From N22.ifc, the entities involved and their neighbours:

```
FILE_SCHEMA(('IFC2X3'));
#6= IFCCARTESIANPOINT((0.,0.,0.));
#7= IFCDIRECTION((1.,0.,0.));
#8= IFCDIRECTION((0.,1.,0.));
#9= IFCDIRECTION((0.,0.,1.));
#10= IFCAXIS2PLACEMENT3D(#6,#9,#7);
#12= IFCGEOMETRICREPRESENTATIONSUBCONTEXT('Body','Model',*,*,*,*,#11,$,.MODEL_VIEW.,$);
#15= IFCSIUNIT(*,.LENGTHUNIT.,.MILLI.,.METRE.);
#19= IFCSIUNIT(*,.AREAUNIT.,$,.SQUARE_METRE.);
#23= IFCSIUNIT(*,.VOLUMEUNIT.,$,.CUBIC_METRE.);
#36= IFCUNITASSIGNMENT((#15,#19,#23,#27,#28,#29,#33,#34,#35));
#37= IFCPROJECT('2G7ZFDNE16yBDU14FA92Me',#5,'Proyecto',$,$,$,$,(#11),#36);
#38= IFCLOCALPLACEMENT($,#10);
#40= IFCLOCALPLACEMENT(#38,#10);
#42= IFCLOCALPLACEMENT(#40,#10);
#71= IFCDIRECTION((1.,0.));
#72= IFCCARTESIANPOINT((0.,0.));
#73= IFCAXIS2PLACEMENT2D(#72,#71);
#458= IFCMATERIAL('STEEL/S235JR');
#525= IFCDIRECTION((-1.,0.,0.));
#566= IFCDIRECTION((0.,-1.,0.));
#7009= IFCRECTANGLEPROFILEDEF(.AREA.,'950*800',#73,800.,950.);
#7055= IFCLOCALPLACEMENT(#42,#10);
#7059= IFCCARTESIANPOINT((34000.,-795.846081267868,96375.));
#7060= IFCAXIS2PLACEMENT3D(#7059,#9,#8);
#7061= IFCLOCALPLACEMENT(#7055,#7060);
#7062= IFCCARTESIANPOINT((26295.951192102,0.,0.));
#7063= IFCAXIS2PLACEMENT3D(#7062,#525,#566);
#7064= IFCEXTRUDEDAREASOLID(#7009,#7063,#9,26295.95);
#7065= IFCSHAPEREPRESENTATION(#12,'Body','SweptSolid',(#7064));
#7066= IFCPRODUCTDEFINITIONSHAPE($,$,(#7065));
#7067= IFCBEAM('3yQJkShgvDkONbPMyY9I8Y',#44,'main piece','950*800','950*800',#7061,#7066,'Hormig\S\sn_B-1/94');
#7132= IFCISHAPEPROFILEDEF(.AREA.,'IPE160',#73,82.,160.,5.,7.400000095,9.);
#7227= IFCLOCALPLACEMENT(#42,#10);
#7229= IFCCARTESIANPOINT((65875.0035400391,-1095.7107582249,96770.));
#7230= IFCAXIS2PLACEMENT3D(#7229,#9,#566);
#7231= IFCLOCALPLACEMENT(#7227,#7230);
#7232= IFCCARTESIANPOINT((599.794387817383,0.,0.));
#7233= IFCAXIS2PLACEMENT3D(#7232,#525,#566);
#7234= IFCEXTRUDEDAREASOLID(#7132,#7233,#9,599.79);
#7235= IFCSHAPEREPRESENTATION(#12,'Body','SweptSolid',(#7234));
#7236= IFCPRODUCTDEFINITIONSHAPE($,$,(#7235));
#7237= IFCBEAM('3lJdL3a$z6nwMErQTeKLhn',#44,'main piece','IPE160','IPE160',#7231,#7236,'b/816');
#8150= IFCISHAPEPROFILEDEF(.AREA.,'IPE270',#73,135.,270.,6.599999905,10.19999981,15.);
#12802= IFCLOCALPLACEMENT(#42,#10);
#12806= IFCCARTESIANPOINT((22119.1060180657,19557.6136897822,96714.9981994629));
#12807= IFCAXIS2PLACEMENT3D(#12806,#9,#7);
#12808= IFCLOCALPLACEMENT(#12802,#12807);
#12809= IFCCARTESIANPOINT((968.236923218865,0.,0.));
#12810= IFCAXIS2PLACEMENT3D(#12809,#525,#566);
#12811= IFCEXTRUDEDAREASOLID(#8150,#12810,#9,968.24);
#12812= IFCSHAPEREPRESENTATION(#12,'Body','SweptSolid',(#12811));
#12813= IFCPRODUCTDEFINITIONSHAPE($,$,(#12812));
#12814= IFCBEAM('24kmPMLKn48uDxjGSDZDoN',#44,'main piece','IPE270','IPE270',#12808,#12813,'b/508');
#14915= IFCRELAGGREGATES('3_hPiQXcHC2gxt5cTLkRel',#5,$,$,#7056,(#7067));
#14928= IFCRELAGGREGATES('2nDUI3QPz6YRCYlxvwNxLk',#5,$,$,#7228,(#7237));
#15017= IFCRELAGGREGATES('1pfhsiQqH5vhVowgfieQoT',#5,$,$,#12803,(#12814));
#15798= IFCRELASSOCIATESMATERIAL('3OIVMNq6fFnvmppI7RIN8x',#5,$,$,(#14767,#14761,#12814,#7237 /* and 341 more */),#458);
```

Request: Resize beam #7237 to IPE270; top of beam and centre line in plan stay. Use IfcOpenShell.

```python
import ifcopenshell
import ifcopenshell.util.element
import ifcopenshell.util.representation

model = ifcopenshell.open("N22.ifc")

member = model.by_guid("3lJdL3a$z6nwMErQTeKLhn")
source = next(p for p in model.by_type("IfcIShapeProfileDef") if p.ProfileName == "IPE270")

body = ifcopenshell.util.representation.get_representation(member, "Model", "Body")
solid = body.Items[0]
old_profile = solid.SweptArea

# Copy the section's sizes but keep this member's own profile position.
profile = ifcopenshell.util.element.copy(model, source)
# Profiles are centred, so shift by half the change in depth to hold the top.
shift = (old_profile.OverallDepth - profile.OverallDepth) / 2
x, y = old_profile.Position.Location.Coordinates
up = (0.0, 1.0)  # upwards, in the solid's own plane
location = model.createIfcCartesianPoint((x + up[0] * shift, y + up[1] * shift))
profile.Position = model.createIfcAxis2Placement2D(location, old_profile.Position.RefDirection)
solid.SweptArea = profile
if not model.get_total_inverses(old_profile):
    ifcopenshell.util.element.remove_deep2(model, old_profile)
member.Description = member.Description.replace("IPE160", "IPE270")
member.ObjectType = member.ObjectType.replace("IPE160", "IPE270")

print(solid.SweptArea)

model.write("N22-out.ifc")
```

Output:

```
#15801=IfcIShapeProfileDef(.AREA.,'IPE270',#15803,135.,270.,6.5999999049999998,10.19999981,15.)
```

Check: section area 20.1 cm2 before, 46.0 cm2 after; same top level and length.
